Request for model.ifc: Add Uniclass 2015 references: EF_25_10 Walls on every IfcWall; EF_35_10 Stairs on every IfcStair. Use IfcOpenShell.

First a look at what the model holds.

```python
import ifcopenshell

model = ifcopenshell.open("model.ifc")
print(model.schema)
print("classifications:", [c.Name for c in model.by_type("IfcClassification")])
for ifc_class in ("IfcDoor", "IfcRoof", "IfcStair", "IfcWall", "IfcWindow"):
    print(ifc_class, len(model.by_type(ifc_class)))
```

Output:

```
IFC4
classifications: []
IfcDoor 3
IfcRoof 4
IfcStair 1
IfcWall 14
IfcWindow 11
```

```python
import ifcopenshell
import ifcopenshell.api.classification

model = ifcopenshell.open("model.ifc")

system = ifcopenshell.api.classification.add_classification(model, classification="Uniclass 2015")

codes = {
    "IfcWall": ("EF_25_10", "Walls"),
    "IfcStair": ("EF_35_10", "Stairs"),
}
for ifc_class, (code, name) in codes.items():
    products = model.by_type(ifc_class)
    ifcopenshell.api.classification.add_reference(
        model, products=products, classification=system, identification=code, name=name
    )
    print(code, len(products))

model.write("model_updated.ifc")
```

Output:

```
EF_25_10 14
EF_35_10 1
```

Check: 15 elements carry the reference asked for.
